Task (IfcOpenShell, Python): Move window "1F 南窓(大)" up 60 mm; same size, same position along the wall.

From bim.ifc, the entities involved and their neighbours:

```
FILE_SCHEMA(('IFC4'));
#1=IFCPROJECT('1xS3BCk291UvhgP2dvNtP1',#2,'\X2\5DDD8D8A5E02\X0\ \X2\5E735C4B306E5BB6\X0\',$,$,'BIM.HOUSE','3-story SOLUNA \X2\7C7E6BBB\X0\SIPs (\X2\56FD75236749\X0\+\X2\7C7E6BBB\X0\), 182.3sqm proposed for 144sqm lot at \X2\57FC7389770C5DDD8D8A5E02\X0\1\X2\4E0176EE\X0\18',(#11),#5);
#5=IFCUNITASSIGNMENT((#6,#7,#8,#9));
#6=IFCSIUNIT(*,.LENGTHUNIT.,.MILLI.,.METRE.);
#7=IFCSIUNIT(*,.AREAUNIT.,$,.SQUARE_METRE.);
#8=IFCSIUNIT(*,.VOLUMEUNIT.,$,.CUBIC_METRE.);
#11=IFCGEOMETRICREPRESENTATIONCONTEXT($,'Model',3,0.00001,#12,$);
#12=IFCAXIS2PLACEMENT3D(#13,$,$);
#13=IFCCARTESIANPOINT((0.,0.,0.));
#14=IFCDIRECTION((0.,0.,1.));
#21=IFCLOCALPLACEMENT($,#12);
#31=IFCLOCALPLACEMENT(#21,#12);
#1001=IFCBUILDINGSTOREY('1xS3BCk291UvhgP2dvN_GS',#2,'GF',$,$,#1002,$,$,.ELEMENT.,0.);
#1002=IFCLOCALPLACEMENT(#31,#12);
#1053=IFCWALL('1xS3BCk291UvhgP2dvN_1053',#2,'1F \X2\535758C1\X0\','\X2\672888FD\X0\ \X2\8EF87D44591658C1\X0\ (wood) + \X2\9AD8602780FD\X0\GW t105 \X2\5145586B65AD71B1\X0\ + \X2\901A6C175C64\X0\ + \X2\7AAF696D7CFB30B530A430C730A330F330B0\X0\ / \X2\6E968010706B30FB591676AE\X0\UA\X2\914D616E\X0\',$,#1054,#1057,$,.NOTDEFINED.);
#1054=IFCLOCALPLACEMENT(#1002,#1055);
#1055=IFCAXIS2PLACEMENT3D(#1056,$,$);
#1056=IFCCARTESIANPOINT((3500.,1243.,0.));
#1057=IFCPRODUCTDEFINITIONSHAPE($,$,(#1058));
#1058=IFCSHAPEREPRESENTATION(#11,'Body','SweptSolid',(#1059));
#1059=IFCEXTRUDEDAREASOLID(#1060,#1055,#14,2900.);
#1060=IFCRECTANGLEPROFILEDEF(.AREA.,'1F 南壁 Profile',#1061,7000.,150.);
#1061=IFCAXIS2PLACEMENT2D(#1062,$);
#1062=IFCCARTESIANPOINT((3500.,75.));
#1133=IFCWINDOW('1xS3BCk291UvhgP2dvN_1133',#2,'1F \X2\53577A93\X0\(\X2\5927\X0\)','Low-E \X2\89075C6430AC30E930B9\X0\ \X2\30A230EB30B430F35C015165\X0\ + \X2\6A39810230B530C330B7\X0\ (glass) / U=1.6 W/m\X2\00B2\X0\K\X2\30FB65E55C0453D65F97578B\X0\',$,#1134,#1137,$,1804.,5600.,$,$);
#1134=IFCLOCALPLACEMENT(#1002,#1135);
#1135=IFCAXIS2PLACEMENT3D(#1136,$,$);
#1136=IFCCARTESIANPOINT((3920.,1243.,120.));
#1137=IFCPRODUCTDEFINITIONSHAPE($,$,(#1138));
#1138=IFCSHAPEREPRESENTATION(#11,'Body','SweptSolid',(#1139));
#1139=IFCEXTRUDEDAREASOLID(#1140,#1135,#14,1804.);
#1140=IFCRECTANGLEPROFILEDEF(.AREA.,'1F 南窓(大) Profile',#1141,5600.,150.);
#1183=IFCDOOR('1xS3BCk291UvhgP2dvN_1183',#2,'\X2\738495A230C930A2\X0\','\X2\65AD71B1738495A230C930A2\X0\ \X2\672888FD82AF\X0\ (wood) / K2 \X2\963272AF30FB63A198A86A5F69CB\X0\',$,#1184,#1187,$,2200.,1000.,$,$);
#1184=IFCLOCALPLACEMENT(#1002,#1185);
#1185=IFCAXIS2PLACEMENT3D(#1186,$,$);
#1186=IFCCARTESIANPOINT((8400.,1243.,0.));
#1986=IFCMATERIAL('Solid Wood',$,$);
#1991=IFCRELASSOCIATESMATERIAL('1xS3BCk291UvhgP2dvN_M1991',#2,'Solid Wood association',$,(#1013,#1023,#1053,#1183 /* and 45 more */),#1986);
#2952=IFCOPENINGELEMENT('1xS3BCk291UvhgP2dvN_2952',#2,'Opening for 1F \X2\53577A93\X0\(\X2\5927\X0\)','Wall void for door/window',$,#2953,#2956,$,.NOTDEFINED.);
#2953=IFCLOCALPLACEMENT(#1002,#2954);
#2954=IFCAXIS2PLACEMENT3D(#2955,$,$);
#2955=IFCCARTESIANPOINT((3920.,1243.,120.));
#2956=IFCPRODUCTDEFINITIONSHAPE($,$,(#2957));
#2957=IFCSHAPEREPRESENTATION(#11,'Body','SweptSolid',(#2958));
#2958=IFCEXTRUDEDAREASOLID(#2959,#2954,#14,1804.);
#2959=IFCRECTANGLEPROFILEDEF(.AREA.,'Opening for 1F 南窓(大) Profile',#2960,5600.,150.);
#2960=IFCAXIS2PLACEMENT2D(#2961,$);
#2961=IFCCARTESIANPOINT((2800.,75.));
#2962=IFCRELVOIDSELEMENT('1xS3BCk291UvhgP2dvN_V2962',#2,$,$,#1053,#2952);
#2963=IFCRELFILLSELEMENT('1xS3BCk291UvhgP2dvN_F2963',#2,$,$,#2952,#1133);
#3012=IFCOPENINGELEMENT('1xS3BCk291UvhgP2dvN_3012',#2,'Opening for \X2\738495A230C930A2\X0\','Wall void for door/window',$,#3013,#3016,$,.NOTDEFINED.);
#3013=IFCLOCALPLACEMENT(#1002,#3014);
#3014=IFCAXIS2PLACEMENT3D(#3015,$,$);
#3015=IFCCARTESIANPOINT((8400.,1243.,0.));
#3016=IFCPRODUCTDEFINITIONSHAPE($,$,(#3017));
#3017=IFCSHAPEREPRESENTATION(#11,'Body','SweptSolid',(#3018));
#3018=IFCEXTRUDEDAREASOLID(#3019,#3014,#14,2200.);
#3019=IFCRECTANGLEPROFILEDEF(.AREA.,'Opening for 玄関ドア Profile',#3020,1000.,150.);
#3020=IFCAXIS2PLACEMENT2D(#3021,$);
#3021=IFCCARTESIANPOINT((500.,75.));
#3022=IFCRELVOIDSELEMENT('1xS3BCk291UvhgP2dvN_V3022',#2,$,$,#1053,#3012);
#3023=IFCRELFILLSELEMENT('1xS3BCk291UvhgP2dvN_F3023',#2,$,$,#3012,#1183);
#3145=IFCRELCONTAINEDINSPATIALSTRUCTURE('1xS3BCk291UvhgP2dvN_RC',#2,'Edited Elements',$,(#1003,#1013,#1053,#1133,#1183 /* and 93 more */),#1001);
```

```python
import numpy as np
import ifcopenshell
import ifcopenshell.api.geometry
import ifcopenshell.util.placement
import ifcopenshell.util.unit

model = ifcopenshell.open("bim.ifc")
unit_scale = ifcopenshell.util.unit.calculate_unit_scale(model)

window = model.by_guid("1xS3BCk291UvhgP2dvN_1133")
opening = window.FillsVoids[0].RelatingOpeningElement
dz = 0.06 / unit_scale

shift = np.array([0.0, 0.0, dz])
# The window is not placed relative to its opening, so move both.
for product in (opening, window):
    matrix = ifcopenshell.util.placement.get_local_placement(product.ObjectPlacement)
    matrix[:3, 3] += shift
    ifcopenshell.api.geometry.edit_object_placement(model, product=product, matrix=matrix, is_si=False)

print(f"moved by {dz * unit_scale:+.3f} m")

model.write("bim-out.ifc")
```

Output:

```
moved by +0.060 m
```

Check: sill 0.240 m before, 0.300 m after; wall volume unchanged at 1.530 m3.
